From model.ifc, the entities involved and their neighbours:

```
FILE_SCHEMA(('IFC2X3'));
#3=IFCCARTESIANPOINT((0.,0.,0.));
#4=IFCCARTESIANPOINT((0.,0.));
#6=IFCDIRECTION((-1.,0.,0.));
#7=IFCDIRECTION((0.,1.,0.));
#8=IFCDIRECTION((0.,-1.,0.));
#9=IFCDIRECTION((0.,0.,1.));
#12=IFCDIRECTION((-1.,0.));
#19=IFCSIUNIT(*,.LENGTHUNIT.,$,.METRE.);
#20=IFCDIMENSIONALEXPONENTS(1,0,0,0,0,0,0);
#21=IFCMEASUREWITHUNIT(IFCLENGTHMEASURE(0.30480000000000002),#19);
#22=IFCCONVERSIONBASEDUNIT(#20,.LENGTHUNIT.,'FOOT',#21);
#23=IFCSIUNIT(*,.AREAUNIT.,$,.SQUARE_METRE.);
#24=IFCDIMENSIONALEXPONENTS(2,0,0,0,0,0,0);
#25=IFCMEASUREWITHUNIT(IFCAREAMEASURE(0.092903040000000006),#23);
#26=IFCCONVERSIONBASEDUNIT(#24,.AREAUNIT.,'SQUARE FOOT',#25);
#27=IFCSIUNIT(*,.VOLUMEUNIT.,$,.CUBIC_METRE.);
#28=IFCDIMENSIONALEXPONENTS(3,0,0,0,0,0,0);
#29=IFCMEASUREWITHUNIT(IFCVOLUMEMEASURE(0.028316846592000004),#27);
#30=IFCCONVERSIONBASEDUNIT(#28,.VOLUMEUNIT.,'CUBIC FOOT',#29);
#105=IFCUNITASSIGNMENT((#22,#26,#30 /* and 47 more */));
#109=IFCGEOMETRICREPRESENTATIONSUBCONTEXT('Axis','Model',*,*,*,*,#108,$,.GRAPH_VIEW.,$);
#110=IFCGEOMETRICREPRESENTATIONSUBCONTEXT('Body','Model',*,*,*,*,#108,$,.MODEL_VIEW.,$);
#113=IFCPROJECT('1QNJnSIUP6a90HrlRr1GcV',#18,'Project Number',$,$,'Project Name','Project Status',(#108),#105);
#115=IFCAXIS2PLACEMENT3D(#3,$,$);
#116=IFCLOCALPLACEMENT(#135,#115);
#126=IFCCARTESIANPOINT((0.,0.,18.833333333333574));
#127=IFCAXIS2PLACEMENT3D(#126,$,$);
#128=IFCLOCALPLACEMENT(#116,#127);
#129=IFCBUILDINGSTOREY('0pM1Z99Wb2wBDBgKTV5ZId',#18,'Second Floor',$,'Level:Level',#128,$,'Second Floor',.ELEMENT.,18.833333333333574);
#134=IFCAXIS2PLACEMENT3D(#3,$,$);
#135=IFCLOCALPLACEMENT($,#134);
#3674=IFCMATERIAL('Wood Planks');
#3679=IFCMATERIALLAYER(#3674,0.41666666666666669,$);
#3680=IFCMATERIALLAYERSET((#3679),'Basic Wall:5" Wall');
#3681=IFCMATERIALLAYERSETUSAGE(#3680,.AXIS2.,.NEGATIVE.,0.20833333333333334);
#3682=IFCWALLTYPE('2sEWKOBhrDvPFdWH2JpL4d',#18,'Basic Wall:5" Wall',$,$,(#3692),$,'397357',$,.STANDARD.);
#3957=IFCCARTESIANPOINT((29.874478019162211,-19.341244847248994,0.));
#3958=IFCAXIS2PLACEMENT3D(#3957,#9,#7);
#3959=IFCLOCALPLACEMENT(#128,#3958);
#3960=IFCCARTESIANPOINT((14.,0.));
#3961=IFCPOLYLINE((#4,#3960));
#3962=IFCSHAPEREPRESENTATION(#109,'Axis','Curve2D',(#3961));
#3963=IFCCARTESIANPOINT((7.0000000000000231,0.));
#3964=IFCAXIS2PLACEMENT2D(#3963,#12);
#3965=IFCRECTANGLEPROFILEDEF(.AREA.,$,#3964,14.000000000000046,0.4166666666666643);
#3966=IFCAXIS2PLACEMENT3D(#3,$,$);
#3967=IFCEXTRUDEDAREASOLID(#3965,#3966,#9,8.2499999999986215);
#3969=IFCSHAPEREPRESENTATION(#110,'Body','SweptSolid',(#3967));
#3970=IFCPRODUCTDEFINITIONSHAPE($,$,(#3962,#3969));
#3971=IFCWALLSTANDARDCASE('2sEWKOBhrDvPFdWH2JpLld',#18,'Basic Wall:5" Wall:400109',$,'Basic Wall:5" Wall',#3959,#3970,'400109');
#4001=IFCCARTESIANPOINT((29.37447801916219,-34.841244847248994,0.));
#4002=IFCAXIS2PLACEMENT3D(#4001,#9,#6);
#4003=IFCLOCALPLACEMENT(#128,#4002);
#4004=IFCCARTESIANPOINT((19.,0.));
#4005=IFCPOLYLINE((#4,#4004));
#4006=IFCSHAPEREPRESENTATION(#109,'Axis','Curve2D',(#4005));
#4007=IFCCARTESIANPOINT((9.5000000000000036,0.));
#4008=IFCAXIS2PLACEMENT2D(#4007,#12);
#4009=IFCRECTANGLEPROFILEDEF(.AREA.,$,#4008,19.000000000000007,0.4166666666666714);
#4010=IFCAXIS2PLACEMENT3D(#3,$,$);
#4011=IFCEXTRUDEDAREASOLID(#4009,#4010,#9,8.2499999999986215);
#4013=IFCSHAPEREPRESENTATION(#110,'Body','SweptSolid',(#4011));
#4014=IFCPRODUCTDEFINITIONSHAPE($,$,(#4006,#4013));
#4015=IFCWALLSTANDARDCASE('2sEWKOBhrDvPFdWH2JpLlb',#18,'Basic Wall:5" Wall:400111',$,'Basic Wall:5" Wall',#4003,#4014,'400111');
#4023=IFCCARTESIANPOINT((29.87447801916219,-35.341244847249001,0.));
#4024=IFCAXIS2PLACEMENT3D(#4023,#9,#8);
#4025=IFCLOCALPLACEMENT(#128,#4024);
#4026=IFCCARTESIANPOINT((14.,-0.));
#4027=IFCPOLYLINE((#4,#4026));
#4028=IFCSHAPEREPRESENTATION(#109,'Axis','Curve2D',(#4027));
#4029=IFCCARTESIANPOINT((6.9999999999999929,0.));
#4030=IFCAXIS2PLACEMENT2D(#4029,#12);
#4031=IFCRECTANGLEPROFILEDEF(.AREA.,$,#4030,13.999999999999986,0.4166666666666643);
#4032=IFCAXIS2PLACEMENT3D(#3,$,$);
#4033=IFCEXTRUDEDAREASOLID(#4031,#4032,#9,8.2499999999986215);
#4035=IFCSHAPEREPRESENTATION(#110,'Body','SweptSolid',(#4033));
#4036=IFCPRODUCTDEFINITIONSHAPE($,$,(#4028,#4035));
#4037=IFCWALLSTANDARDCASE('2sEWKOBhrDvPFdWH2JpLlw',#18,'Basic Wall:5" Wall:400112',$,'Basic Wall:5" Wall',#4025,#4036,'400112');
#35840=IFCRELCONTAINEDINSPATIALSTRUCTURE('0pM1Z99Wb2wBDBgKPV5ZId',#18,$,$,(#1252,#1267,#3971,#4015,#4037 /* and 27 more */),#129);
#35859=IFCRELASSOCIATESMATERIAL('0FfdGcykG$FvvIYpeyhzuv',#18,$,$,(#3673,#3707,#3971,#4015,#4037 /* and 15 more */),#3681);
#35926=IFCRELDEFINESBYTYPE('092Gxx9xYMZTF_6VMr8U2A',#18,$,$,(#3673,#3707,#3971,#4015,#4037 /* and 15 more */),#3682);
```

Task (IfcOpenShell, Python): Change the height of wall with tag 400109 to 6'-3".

```python
import ifcopenshell
import ifcopenshell.geom
import ifcopenshell.util.representation
import ifcopenshell.util.shape
import ifcopenshell.util.unit

model = ifcopenshell.open("model.ifc")
unit_scale = ifcopenshell.util.unit.calculate_unit_scale(model)
settings = ifcopenshell.geom.settings()


def volume(element):
    """Net volume in cubic metres, openings subtracted."""
    shape = ifcopenshell.geom.create_shape(settings, element)
    return ifcopenshell.util.shape.get_volume(shape.geometry)


wall = model.by_guid("2sEWKOBhrDvPFdWH2JpLld")
before = volume(wall)

body = ifcopenshell.util.representation.get_representation(wall, "Model", "Body")
solid = body.Items[0]
old_height = solid.Depth
solid.Depth = 75 * 0.0254 / unit_scale
after = volume(wall)

print(f"height {old_height:g} -> {solid.Depth:g}, volume {before:.3f} -> {after:.3f} m3")

model.write("model_rev.ifc")
```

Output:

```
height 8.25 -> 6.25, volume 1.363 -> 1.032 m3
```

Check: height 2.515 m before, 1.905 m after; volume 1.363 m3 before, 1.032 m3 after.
